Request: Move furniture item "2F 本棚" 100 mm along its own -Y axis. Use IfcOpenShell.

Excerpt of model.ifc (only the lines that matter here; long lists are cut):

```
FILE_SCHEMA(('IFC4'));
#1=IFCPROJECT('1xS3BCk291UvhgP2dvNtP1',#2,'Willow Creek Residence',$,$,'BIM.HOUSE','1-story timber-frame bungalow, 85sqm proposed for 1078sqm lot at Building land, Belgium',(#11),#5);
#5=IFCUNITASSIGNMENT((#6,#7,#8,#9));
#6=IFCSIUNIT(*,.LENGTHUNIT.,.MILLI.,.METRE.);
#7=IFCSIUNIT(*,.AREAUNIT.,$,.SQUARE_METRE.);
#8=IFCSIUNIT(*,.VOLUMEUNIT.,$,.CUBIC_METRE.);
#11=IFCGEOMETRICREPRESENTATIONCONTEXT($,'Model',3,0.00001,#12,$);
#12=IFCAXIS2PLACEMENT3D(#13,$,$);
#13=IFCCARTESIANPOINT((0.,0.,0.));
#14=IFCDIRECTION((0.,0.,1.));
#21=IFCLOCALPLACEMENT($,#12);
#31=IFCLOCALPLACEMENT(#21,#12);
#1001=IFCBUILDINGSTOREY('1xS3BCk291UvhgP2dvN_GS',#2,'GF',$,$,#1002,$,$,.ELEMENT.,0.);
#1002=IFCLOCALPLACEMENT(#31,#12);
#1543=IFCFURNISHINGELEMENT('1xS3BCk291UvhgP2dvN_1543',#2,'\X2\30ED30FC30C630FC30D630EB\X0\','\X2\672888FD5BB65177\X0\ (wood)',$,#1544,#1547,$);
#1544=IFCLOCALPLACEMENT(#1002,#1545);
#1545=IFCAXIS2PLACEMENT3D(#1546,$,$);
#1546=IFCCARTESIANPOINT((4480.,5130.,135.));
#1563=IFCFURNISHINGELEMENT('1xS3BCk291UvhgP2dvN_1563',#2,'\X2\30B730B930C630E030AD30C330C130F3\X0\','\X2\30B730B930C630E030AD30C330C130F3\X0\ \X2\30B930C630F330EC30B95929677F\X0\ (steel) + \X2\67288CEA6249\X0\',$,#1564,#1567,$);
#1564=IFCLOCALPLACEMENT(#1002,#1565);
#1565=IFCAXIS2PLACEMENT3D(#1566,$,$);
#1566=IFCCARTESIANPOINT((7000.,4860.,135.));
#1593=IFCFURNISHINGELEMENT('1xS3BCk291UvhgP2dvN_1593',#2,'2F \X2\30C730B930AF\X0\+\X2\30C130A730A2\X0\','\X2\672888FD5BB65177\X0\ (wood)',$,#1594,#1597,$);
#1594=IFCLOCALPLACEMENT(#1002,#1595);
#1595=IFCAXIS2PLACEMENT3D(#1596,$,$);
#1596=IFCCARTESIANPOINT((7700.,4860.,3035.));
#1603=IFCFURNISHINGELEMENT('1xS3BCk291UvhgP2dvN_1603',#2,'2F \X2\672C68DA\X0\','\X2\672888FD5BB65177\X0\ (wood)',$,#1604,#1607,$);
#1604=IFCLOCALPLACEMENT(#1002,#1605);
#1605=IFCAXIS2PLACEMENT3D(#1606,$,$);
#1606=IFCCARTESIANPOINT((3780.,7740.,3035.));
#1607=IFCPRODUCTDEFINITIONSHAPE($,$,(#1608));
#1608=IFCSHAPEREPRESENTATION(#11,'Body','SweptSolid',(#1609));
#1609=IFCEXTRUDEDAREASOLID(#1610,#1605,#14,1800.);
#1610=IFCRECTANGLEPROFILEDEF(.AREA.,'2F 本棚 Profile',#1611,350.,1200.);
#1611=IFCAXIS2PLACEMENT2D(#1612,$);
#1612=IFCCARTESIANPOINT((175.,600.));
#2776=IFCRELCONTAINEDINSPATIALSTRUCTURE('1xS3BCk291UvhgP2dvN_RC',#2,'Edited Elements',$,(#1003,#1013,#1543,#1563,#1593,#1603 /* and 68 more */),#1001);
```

```python
import ifcopenshell
import ifcopenshell.api.geometry
import ifcopenshell.util.placement

model = ifcopenshell.open("model.ifc")

item = model.by_guid("1xS3BCk291UvhgP2dvN_1603")
matrix = ifcopenshell.util.placement.get_local_placement(item.ObjectPlacement)
matrix[:3, 3] -= matrix[:3, 1] * 100.0
ifcopenshell.api.geometry.edit_object_placement(model, product=item, matrix=matrix, is_si=False)

print(ifcopenshell.util.placement.get_local_placement(item.ObjectPlacement).round(3) + 0.0)

model.write("model_v2.ifc")
```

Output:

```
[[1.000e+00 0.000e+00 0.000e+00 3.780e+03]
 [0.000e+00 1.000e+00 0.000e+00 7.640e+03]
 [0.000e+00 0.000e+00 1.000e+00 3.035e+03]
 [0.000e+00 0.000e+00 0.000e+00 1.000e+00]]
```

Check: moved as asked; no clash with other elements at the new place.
